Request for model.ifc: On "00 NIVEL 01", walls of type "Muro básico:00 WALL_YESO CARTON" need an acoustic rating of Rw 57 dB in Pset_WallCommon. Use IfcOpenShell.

First a look at what the model holds.

```python
import ifcopenshell
import ifcopenshell.util.element

model = ifcopenshell.open("model.ifc")
print(model.schema)
storey = next(s for s in model.by_type("IfcBuildingStorey") if s.Name == "00 NIVEL 01")
walls = [e for e in ifcopenshell.util.element.get_decomposition(storey) if e.is_a("IfcWall")]
seen = {}
for e in walls:
    element_type = ifcopenshell.util.element.get_type(e)
    key = (element_type.Name if element_type != e and element_type else None, ifcopenshell.util.element.get_pset(e, "Pset_WallCommon", "AcousticRating"))
    seen[key] = seen.get(key, 0) + 1
for (name, value), count in sorted(seen.items(), key=str):
    print(count, "x", name, "|", value)
```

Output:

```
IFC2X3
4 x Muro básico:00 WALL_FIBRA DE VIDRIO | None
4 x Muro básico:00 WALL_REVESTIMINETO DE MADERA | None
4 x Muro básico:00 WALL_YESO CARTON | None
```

```python
import ifcopenshell
import ifcopenshell.api.pset
import ifcopenshell.util.element

model = ifcopenshell.open("model.ifc")

storey = next(s for s in model.by_type("IfcBuildingStorey") if s.Name == "00 NIVEL 01")
walls = [e for e in ifcopenshell.util.element.get_decomposition(storey) if e.is_a("IfcWall")]

count = 0
for e in walls:
    element_type = ifcopenshell.util.element.get_type(e)
    if element_type in (None, e) or element_type.Name != "Muro básico:00 WALL_YESO CARTON":
        continue
    # add_pset returns the element's existing set when there is one.
    pset = ifcopenshell.api.pset.add_pset(model, product=e, name="Pset_WallCommon")
    ifcopenshell.api.pset.edit_pset(model, pset=pset, properties={"AcousticRating": "Rw 57 dB"})
    count += 1

print(count, "walls updated")

model.write("model_v2.ifc")
```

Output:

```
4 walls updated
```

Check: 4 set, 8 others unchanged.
